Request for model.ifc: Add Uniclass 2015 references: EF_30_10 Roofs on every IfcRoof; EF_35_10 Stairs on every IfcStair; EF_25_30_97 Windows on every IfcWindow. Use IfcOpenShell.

First a look at what the model holds.

```python
import ifcopenshell

model = ifcopenshell.open("model.ifc")
print(model.schema)
print("classifications:", [c.Name for c in model.by_type("IfcClassification")])
for ifc_class in ("IfcDoor", "IfcRoof", "IfcStair", "IfcWall", "IfcWindow"):
    print(ifc_class, len(model.by_type(ifc_class)))
```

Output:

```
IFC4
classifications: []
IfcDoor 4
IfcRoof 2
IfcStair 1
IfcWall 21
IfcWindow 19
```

```python
import ifcopenshell
import ifcopenshell.api.classification

model = ifcopenshell.open("model.ifc")

system = ifcopenshell.api.classification.add_classification(model, classification="Uniclass 2015")

codes = {
    "IfcRoof": ("EF_30_10", "Roofs"),
    "IfcStair": ("EF_35_10", "Stairs"),
    "IfcWindow": ("EF_25_30_97", "Windows"),
}
for ifc_class, (code, name) in codes.items():
    products = model.by_type(ifc_class)
    ifcopenshell.api.classification.add_reference(
        model, products=products, classification=system, identification=code, name=name
    )
    print(code, len(products))

model.write("model_v2.ifc")
```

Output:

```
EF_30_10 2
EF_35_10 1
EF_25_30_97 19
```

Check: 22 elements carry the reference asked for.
